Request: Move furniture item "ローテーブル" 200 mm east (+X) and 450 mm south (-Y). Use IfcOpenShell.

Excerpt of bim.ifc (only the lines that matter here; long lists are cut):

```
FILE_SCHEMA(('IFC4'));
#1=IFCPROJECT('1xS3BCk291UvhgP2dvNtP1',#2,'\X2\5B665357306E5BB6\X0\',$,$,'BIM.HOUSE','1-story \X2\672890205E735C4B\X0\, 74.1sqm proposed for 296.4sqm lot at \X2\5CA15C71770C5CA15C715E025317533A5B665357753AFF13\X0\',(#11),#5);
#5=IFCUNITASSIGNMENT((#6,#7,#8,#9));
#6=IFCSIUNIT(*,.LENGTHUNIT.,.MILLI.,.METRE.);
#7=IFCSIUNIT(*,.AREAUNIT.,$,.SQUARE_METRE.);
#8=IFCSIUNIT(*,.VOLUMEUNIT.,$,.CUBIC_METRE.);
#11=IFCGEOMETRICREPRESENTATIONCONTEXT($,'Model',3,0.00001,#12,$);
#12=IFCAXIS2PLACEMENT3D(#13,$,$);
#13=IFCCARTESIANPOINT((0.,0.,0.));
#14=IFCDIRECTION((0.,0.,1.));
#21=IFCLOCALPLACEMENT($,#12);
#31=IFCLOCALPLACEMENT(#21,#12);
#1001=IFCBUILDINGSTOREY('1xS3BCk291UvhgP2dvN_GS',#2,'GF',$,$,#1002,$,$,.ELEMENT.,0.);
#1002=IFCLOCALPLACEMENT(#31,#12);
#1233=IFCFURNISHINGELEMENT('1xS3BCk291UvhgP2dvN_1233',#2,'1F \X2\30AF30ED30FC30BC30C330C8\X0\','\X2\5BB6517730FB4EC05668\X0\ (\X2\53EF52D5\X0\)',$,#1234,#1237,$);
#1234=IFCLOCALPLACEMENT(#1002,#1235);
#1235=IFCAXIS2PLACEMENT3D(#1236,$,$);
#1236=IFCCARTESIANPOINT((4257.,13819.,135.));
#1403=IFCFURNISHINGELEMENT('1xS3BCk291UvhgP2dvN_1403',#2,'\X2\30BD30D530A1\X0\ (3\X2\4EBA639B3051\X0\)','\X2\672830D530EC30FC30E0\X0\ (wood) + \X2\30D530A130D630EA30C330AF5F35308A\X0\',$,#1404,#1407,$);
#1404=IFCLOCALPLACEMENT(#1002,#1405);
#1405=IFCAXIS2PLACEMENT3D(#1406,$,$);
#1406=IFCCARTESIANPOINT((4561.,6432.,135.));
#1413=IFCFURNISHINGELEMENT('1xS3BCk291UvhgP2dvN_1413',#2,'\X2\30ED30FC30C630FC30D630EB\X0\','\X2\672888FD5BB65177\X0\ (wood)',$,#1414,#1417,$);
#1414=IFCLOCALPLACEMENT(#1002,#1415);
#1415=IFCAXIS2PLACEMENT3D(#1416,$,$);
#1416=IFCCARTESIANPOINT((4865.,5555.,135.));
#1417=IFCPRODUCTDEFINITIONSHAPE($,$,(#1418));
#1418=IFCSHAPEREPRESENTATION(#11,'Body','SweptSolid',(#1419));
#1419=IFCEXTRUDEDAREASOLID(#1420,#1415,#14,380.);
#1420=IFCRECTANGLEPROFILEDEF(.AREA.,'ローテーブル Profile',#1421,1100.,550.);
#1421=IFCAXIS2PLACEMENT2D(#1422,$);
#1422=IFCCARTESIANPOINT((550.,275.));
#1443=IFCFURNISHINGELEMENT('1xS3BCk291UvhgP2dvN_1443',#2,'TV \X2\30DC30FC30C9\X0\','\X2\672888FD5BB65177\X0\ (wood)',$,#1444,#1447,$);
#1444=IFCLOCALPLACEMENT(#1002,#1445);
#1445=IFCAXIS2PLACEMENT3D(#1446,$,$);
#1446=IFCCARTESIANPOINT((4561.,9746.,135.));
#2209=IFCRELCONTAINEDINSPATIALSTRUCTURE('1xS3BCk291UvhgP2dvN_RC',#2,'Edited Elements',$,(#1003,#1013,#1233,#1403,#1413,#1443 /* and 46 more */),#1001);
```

```python
import ifcopenshell
import ifcopenshell.api.geometry
import ifcopenshell.util.placement
import ifcopenshell.util.unit

model = ifcopenshell.open("bim.ifc")
unit_scale = ifcopenshell.util.unit.calculate_unit_scale(model)

item = model.by_guid("1xS3BCk291UvhgP2dvN_1413")
matrix = ifcopenshell.util.placement.get_local_placement(item.ObjectPlacement)
matrix[0, 3] += 0.2 / unit_scale
matrix[1, 3] -= 0.45 / unit_scale
ifcopenshell.api.geometry.edit_object_placement(model, product=item, matrix=matrix, is_si=False)

print(ifcopenshell.util.placement.get_local_placement(item.ObjectPlacement).round(3) + 0.0)

model.write("bim_edited.ifc")
```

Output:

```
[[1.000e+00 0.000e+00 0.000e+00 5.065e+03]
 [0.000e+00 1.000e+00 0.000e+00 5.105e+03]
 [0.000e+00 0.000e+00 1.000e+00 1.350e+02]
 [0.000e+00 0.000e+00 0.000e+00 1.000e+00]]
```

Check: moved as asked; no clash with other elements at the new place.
